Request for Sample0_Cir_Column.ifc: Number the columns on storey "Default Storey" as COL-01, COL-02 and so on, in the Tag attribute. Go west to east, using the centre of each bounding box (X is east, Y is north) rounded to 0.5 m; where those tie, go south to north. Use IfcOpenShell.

First a look at what the model holds.

```python
import ifcopenshell
import ifcopenshell.util.element
import ifcopenshell.util.placement

model = ifcopenshell.open("Sample0_Cir_Column.ifc")
print(model.schema)
storey = next(s for s in model.by_type("IfcBuildingStorey") if s.Name == "Default Storey")
columns = [e for e in ifcopenshell.util.element.get_decomposition(storey) if e.is_a("IfcColumn")]
for e in sorted(columns, key=lambda e: e.id()):
    origin = ifcopenshell.util.placement.get_local_placement(e.ObjectPlacement)[:3, 3]
    print(e.id(), e.Tag, e.Name, origin.round(2) + 0.0, sep=" | ")
```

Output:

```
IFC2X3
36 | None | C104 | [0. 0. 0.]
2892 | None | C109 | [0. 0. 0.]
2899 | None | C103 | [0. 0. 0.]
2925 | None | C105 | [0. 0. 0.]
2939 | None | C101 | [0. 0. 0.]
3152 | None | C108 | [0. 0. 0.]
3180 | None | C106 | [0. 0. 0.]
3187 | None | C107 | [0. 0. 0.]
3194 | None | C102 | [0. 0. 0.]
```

```python
import ifcopenshell
import ifcopenshell.geom
import ifcopenshell.util.element
import ifcopenshell.util.shape

model = ifcopenshell.open("Sample0_Cir_Column.ifc")
settings = ifcopenshell.geom.settings()
settings.set("use-world-coords", True)


def centre(element):
    shape = ifcopenshell.geom.create_shape(settings, element)
    return ifcopenshell.util.shape.get_bbox_centroid(shape.geometry)


storey = next(s for s in model.by_type("IfcBuildingStorey") if s.Name == "Default Storey")
columns = [e for e in ifcopenshell.util.element.get_decomposition(storey) if e.is_a("IfcColumn")]

# Insertion points can sit at a corner or the storey origin, so sort by the geometry (in metres).
centres = {e: centre(e) for e in columns}
columns.sort(key=lambda e: (round(centres[e][0] / 0.5), centres[e][1]))

for i, e in enumerate(columns, start=1):
    number = f"COL-{i:02d}"
    e.Tag = number
    print(e.id(), number)

model.write("Sample0_Cir_Column_updated.ifc")
```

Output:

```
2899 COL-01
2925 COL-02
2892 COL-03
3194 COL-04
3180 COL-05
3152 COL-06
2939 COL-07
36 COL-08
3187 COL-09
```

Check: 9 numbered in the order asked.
